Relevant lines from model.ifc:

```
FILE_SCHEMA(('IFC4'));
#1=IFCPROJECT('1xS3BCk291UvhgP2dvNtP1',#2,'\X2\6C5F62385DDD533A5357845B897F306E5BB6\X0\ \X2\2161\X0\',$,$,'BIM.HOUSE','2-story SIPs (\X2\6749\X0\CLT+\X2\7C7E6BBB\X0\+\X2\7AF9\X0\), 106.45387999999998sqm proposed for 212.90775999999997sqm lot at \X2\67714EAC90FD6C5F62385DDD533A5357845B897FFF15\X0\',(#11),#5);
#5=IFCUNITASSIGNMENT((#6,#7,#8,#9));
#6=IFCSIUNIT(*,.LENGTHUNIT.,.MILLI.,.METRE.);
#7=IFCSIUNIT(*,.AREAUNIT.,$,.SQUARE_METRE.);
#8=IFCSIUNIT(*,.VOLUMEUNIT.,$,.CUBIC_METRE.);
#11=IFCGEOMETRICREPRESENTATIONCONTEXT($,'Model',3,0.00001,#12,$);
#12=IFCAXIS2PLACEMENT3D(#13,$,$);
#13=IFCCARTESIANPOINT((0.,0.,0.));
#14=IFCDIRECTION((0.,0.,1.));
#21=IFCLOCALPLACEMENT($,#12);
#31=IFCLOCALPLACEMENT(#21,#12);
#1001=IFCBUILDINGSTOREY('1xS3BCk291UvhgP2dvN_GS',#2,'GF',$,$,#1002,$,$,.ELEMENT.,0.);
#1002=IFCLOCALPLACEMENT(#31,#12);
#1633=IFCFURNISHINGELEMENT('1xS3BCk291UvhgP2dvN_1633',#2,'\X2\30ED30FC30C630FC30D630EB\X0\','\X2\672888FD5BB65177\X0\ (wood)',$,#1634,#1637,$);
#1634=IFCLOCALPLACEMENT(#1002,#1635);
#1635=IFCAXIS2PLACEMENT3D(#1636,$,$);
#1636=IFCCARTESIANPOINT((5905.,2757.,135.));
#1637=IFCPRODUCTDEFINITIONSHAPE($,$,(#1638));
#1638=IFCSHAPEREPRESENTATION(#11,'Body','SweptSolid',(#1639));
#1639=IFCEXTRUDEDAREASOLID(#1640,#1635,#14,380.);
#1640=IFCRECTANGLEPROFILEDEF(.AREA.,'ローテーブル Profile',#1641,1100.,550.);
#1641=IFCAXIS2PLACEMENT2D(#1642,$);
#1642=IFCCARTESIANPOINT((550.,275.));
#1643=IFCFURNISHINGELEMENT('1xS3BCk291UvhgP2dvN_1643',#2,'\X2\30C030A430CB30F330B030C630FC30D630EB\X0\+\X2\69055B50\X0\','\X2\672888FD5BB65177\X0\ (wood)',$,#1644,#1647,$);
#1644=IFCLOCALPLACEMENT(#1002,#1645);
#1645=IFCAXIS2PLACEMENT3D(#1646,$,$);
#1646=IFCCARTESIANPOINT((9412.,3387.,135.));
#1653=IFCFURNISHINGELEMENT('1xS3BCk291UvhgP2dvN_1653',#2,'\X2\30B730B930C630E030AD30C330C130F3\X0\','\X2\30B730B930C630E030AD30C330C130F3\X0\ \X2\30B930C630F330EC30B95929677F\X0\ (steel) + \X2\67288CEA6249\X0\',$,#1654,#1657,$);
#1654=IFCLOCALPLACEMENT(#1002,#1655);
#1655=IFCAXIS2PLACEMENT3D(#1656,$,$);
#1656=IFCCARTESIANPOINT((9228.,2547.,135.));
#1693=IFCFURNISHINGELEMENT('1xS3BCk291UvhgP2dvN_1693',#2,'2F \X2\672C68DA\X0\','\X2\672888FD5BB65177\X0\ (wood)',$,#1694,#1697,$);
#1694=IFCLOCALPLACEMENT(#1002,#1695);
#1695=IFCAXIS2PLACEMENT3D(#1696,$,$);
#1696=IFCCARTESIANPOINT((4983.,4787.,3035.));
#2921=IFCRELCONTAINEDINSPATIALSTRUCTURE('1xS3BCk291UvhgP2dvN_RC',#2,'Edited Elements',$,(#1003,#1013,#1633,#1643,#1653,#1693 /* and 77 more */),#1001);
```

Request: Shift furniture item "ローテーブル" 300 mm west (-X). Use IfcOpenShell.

```python
import ifcopenshell
import ifcopenshell.api.geometry
import ifcopenshell.util.placement

model = ifcopenshell.open("model.ifc")

item = model.by_id(1633)
matrix = ifcopenshell.util.placement.get_local_placement(item.ObjectPlacement)
matrix[0, 3] -= 300.0
ifcopenshell.api.geometry.edit_object_placement(model, product=item, matrix=matrix, is_si=False)

print(ifcopenshell.util.placement.get_local_placement(item.ObjectPlacement).round(3) + 0.0)

model.write("model-out.ifc")
```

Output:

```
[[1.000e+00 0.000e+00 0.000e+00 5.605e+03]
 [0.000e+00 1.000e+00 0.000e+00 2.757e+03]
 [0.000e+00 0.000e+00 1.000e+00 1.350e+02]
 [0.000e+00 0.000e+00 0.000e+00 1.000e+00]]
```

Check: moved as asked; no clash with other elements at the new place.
